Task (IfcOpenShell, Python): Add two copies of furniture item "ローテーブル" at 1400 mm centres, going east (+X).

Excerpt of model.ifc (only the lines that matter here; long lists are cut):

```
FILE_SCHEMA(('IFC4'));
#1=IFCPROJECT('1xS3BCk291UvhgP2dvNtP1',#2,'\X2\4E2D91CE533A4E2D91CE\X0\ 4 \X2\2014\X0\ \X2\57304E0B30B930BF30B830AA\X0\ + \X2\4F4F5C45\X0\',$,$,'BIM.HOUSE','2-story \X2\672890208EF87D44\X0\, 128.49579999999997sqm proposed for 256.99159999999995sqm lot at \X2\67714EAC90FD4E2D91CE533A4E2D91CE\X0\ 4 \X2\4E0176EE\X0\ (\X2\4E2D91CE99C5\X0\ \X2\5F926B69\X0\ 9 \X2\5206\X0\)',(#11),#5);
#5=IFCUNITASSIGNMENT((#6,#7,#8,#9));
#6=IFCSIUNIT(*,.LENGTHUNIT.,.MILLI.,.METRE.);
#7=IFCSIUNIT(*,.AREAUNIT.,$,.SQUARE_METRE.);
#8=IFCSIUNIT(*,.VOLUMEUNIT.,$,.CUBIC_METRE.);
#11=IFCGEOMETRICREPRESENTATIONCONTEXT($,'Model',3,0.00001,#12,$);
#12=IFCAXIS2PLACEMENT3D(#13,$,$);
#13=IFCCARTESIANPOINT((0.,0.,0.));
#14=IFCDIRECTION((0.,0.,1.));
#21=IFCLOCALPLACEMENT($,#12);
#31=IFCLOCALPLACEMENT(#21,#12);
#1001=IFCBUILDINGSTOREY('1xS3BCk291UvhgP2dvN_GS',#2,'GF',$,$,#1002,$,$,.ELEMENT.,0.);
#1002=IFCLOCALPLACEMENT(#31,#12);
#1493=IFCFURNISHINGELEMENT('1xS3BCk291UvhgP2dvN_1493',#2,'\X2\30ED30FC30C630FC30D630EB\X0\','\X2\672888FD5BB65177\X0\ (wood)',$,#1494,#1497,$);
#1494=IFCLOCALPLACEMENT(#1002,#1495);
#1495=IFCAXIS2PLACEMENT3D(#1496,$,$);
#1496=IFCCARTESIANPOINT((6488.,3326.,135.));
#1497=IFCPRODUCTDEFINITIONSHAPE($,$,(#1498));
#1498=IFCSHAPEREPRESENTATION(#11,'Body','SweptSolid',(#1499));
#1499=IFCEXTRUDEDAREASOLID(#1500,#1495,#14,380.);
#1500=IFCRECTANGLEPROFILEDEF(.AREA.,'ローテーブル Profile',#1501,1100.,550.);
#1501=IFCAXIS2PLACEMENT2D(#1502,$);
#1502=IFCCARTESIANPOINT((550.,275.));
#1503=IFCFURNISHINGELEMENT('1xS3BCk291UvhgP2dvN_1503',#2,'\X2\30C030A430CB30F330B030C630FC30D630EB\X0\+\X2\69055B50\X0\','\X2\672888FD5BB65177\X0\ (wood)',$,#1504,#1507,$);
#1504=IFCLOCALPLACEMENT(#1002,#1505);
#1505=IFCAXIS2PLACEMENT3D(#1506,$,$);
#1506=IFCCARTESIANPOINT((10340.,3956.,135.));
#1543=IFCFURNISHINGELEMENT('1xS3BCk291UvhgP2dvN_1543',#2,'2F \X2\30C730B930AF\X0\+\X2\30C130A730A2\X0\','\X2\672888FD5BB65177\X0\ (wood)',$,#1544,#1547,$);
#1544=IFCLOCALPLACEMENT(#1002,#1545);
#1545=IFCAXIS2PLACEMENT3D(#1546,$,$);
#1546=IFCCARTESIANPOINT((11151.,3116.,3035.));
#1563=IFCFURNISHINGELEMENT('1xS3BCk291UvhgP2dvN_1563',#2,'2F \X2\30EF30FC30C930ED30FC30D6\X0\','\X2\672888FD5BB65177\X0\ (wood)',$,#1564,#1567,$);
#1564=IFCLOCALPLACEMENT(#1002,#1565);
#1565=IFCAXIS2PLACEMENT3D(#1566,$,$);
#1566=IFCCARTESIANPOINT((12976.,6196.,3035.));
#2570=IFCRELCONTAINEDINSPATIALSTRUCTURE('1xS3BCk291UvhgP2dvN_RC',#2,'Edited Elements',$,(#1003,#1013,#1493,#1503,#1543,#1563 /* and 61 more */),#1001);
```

```python
import numpy as np
import ifcopenshell
import ifcopenshell.api.geometry
import ifcopenshell.api.root
import ifcopenshell.util.element
import ifcopenshell.util.placement
import ifcopenshell.util.unit

model = ifcopenshell.open("model.ifc")
unit_scale = ifcopenshell.util.unit.calculate_unit_scale(model)


def reuse_history(source, copy):
    """copy_class also copies each property set's owner history, people and application; keep the originals."""
    for rel in copy.IsDefinedBy:
        if rel.is_a("IfcRelDefinesByProperties") and (history := rel.RelatingPropertyDefinition.OwnerHistory):
            rel.RelatingPropertyDefinition.OwnerHistory = source.OwnerHistory
            ifcopenshell.util.element.remove_deep2(model, history)


source = model.by_id(1493)
base = ifcopenshell.util.placement.get_local_placement(source.ObjectPlacement)
step = np.array([1.0, 0.0, 0.0]) * 1.4 / unit_scale

for i in range(1, 3):
    copy = ifcopenshell.api.root.copy_class(model, product=source)
    copy.Representation = ifcopenshell.util.element.copy_deep(
        model, source.Representation, exclude=["IfcGeometricRepresentationContext", "IfcRepresentationMap"]
    )
    reuse_history(source, copy)
    matrix = base.copy()
    matrix[:3, 3] += i * step
    print("added at", matrix[:3, 3].round(3) + 0.0)
    ifcopenshell.api.geometry.edit_object_placement(model, product=copy, matrix=matrix, is_si=False)

model.write("model_v2.ifc")
```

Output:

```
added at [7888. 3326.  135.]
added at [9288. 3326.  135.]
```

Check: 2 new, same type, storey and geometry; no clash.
